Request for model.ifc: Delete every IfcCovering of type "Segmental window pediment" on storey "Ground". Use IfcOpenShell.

First a look at what the model holds.

```python
import ifcopenshell
import ifcopenshell.util.element

model = ifcopenshell.open("model.ifc")
print(model.schema)
storey = next(s for s in model.by_type("IfcBuildingStorey") if s.Name == "Ground")
coverings = [e for e in ifcopenshell.util.element.get_decomposition(storey) if e.is_a("IfcCovering")]
seen = {}
for e in coverings:
    element_type = ifcopenshell.util.element.get_type(e)
    name = element_type.Name if element_type not in (None, e) else None
    seen[name] = seen.get(name, 0) + 1
for name, count in sorted(seen.items(), key=str):
    print(count, "x", name)
```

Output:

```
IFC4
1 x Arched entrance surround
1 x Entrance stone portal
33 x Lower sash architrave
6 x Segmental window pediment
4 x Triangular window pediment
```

```python
import ifcopenshell
import ifcopenshell.api.root
import ifcopenshell.util.element

model = ifcopenshell.open("model.ifc")

storey = next(s for s in model.by_type("IfcBuildingStorey") if s.Name == "Ground")
coverings = [e for e in ifcopenshell.util.element.get_decomposition(storey) if e.is_a("IfcCovering")]
targets = [e for e in coverings if (t := ifcopenshell.util.element.get_type(e)) not in (None, e) and t.Name == "Segmental window pediment"]

for e in targets:
    ifcopenshell.api.root.remove_product(model, product=e)
print(len(targets), "removed")

model.write("model-out.ifc")
```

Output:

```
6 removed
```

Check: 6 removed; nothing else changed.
